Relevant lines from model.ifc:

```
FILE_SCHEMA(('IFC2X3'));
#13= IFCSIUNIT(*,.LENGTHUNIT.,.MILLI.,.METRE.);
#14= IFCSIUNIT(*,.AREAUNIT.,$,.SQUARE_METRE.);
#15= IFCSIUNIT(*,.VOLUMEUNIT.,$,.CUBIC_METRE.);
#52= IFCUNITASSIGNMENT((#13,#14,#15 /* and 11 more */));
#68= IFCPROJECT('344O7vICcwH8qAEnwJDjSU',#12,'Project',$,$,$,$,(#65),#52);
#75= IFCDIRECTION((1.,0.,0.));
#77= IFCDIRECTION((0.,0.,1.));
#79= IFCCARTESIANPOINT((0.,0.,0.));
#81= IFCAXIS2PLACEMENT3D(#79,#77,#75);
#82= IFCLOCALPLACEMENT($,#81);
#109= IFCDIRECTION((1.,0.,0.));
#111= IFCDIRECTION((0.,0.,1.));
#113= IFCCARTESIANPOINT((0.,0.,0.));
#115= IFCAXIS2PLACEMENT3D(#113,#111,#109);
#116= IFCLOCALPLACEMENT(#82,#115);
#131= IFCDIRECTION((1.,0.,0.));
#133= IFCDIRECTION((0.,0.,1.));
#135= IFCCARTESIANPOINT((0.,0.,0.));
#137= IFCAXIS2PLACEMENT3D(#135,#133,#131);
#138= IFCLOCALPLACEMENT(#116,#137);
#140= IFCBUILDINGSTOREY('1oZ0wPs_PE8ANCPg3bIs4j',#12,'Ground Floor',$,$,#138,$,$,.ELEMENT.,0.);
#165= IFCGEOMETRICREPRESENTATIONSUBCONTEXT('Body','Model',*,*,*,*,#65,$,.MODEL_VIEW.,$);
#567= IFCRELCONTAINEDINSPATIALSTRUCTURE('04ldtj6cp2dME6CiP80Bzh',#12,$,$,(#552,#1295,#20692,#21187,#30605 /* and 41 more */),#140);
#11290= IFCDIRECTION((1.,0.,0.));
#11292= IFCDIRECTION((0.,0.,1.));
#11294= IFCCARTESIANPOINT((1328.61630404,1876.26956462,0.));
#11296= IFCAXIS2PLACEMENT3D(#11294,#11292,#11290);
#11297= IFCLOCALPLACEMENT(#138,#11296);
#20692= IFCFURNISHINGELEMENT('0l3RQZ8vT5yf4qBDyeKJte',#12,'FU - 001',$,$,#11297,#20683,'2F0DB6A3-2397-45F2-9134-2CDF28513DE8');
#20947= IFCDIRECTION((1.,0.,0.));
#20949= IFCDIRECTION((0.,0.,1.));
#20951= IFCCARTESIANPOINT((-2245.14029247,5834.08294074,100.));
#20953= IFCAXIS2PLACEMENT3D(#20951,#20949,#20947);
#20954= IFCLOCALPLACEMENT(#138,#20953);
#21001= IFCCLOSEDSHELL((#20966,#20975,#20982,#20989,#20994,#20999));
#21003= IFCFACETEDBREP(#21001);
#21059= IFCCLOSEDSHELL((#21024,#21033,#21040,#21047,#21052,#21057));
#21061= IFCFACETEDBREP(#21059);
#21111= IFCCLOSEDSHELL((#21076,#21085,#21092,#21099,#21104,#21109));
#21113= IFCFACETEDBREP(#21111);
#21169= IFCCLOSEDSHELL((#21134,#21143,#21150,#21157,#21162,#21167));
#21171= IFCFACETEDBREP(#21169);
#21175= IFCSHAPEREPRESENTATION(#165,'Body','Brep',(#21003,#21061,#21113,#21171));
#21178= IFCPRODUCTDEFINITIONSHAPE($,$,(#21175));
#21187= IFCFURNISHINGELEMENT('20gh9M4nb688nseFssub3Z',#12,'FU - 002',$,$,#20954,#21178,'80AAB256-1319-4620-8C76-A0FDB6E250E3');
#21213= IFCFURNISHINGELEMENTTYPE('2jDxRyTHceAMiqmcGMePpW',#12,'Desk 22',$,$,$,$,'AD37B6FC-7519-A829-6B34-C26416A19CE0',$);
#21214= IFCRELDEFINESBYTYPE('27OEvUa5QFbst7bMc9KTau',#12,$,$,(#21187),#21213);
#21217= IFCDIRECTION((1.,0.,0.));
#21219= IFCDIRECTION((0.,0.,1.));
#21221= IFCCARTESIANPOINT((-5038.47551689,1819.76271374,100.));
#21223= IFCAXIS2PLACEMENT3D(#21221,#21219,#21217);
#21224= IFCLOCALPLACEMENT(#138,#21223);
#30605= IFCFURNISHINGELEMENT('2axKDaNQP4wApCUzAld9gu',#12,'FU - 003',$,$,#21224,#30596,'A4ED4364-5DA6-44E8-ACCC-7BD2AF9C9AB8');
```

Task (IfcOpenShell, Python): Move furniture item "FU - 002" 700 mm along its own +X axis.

```python
import ifcopenshell
import ifcopenshell.api.geometry
import ifcopenshell.util.placement

model = ifcopenshell.open("model.ifc")

item = model.by_guid("20gh9M4nb688nseFssub3Z")
matrix = ifcopenshell.util.placement.get_local_placement(item.ObjectPlacement)
matrix[:3, 3] += matrix[:3, 0] * 700.0
ifcopenshell.api.geometry.edit_object_placement(model, product=item, matrix=matrix, is_si=False)

print(ifcopenshell.util.placement.get_local_placement(item.ObjectPlacement).round(3) + 0.0)

model.write("model_v2.ifc")
```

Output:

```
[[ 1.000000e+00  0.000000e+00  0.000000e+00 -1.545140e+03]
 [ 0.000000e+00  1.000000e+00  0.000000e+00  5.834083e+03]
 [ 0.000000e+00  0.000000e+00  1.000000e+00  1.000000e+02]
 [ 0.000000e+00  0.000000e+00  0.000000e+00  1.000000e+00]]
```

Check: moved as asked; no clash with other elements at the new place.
